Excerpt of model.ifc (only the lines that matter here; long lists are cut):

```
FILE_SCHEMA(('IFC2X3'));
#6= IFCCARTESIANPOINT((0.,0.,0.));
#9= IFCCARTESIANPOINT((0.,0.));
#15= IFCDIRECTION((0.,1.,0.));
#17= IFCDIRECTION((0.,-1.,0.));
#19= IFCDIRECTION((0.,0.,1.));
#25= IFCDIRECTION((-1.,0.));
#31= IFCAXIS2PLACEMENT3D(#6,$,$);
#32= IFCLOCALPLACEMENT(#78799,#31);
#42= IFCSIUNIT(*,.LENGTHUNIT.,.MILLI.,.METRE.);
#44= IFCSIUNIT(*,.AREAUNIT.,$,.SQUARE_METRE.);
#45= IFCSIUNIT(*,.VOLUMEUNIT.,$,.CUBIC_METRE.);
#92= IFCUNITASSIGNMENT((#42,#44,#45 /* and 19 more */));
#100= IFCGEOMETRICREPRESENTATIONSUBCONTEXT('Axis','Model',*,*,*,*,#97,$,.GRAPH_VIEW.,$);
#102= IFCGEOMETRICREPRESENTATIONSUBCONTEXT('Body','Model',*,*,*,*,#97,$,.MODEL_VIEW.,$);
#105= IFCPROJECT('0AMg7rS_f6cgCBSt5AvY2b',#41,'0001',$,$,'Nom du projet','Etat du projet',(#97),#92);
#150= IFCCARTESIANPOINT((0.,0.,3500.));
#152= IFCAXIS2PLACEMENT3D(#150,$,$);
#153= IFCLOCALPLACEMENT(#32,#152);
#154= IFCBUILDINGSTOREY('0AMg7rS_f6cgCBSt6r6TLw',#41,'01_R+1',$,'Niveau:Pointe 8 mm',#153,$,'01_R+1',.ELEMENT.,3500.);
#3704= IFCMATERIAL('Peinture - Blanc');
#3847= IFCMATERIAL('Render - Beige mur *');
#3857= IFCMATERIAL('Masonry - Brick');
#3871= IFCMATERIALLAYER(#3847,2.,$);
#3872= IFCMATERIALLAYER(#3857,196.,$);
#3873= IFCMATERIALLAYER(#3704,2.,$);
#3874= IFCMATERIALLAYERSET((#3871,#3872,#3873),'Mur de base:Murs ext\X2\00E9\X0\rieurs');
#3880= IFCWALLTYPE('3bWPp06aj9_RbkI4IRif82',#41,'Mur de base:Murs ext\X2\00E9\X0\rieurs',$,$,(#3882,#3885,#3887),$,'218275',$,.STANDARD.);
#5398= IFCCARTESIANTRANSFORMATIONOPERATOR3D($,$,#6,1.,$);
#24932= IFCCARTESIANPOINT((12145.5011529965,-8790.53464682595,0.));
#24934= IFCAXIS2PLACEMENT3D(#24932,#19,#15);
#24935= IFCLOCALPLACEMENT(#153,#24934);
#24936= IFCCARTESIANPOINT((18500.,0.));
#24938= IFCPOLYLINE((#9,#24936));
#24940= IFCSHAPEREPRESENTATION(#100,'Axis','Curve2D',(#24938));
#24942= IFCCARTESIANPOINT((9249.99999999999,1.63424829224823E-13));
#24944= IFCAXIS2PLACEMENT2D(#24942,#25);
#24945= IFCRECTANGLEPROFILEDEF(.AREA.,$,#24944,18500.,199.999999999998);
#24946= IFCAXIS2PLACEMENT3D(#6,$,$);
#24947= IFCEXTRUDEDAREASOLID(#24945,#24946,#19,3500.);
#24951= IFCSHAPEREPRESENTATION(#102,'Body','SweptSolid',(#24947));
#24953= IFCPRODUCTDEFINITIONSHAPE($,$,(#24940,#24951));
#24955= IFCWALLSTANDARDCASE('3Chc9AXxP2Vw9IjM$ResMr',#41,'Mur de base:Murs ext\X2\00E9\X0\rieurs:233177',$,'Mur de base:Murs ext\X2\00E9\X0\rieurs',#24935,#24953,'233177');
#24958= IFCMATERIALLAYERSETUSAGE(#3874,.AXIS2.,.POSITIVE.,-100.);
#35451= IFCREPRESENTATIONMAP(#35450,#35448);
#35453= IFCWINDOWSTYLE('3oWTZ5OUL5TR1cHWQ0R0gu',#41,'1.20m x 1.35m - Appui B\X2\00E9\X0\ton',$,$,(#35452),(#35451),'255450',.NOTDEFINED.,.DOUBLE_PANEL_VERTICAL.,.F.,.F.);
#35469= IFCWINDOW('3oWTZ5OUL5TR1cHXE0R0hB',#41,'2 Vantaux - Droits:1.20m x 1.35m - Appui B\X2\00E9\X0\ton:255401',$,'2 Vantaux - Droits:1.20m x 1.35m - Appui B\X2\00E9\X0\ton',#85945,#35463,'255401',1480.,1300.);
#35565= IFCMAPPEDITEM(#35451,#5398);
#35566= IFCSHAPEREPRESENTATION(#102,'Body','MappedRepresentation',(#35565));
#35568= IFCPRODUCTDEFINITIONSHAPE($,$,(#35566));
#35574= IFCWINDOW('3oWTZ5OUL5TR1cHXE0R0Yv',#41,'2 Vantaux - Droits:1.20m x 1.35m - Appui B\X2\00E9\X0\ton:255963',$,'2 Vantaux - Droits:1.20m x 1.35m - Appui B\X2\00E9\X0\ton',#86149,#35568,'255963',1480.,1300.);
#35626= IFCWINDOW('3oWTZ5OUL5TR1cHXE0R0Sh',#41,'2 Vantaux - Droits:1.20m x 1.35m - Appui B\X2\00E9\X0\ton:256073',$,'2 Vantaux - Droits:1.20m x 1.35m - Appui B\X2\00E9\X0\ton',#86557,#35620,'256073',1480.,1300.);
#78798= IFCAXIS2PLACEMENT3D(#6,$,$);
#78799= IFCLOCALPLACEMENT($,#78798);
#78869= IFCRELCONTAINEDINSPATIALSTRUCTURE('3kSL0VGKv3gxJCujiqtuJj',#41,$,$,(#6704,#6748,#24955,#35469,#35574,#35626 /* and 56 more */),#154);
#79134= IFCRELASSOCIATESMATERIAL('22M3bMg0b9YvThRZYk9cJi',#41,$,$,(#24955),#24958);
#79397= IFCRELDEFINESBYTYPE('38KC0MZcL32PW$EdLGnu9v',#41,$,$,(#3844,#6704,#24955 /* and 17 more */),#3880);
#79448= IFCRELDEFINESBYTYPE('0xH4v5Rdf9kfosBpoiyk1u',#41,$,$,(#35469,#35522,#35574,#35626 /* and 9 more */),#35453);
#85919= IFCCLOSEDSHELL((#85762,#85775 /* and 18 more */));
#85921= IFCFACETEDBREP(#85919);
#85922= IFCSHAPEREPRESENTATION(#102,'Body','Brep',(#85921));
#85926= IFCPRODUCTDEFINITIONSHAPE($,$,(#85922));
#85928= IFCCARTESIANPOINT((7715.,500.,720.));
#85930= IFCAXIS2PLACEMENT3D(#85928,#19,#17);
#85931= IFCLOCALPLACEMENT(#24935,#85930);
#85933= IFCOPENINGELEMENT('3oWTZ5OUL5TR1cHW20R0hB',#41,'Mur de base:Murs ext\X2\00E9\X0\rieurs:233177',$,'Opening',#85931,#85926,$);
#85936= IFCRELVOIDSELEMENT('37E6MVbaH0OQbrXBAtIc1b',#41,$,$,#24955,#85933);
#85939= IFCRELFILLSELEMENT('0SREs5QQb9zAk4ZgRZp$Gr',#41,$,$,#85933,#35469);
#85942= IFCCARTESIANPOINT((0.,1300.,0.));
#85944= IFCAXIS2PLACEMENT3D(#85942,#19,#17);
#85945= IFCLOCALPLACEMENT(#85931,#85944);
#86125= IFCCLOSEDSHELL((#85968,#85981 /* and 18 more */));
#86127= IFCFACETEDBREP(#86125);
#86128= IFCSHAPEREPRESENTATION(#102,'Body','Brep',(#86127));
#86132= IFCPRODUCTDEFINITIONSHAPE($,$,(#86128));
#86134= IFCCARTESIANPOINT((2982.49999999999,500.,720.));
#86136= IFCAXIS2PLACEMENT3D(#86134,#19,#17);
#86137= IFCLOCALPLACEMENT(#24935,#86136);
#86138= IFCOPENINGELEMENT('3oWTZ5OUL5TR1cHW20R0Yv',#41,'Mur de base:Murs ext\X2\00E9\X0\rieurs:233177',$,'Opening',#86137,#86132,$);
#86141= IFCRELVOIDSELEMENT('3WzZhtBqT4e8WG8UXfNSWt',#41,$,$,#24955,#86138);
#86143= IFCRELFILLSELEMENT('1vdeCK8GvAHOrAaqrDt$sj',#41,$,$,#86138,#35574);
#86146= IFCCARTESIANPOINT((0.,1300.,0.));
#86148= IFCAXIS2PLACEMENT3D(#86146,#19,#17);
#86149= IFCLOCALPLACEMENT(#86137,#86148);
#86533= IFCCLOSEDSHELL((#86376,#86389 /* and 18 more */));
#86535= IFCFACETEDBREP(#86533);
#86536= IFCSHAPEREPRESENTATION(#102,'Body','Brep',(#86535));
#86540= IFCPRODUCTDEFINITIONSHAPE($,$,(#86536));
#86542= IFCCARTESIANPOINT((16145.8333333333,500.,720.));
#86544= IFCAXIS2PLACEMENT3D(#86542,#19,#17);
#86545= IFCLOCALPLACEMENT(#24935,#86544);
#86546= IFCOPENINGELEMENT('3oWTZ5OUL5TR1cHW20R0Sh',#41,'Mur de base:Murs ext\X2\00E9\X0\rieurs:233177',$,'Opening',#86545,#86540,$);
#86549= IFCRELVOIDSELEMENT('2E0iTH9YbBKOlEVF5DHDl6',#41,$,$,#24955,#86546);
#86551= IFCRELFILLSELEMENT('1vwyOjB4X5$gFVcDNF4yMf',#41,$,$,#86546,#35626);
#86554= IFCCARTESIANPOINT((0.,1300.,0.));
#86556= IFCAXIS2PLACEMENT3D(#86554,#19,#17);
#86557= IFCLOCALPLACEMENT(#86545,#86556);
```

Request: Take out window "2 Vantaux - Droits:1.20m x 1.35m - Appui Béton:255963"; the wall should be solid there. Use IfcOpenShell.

```python
import ifcopenshell
import ifcopenshell.api.feature
import ifcopenshell.api.root
import ifcopenshell.geom
import ifcopenshell.util.shape

model = ifcopenshell.open("model.ifc")
settings = ifcopenshell.geom.settings()


def volume(element):
    """Net volume in cubic metres, openings subtracted."""
    shape = ifcopenshell.geom.create_shape(settings, element)
    return ifcopenshell.util.shape.get_volume(shape.geometry)


window = model.by_id(35574)
opening = window.FillsVoids[0].RelatingOpeningElement
wall = opening.VoidsElements[0].RelatingBuildingElement
before = volume(wall)

ifcopenshell.api.root.remove_product(model, product=window)
ifcopenshell.api.feature.remove_feature(model, feature=opening)

after = volume(wall)

print(f"wall volume {before:.3f} -> {after:.3f} m3")

model.write("model-out.ifc")
```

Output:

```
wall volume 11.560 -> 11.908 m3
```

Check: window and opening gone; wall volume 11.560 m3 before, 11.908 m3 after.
